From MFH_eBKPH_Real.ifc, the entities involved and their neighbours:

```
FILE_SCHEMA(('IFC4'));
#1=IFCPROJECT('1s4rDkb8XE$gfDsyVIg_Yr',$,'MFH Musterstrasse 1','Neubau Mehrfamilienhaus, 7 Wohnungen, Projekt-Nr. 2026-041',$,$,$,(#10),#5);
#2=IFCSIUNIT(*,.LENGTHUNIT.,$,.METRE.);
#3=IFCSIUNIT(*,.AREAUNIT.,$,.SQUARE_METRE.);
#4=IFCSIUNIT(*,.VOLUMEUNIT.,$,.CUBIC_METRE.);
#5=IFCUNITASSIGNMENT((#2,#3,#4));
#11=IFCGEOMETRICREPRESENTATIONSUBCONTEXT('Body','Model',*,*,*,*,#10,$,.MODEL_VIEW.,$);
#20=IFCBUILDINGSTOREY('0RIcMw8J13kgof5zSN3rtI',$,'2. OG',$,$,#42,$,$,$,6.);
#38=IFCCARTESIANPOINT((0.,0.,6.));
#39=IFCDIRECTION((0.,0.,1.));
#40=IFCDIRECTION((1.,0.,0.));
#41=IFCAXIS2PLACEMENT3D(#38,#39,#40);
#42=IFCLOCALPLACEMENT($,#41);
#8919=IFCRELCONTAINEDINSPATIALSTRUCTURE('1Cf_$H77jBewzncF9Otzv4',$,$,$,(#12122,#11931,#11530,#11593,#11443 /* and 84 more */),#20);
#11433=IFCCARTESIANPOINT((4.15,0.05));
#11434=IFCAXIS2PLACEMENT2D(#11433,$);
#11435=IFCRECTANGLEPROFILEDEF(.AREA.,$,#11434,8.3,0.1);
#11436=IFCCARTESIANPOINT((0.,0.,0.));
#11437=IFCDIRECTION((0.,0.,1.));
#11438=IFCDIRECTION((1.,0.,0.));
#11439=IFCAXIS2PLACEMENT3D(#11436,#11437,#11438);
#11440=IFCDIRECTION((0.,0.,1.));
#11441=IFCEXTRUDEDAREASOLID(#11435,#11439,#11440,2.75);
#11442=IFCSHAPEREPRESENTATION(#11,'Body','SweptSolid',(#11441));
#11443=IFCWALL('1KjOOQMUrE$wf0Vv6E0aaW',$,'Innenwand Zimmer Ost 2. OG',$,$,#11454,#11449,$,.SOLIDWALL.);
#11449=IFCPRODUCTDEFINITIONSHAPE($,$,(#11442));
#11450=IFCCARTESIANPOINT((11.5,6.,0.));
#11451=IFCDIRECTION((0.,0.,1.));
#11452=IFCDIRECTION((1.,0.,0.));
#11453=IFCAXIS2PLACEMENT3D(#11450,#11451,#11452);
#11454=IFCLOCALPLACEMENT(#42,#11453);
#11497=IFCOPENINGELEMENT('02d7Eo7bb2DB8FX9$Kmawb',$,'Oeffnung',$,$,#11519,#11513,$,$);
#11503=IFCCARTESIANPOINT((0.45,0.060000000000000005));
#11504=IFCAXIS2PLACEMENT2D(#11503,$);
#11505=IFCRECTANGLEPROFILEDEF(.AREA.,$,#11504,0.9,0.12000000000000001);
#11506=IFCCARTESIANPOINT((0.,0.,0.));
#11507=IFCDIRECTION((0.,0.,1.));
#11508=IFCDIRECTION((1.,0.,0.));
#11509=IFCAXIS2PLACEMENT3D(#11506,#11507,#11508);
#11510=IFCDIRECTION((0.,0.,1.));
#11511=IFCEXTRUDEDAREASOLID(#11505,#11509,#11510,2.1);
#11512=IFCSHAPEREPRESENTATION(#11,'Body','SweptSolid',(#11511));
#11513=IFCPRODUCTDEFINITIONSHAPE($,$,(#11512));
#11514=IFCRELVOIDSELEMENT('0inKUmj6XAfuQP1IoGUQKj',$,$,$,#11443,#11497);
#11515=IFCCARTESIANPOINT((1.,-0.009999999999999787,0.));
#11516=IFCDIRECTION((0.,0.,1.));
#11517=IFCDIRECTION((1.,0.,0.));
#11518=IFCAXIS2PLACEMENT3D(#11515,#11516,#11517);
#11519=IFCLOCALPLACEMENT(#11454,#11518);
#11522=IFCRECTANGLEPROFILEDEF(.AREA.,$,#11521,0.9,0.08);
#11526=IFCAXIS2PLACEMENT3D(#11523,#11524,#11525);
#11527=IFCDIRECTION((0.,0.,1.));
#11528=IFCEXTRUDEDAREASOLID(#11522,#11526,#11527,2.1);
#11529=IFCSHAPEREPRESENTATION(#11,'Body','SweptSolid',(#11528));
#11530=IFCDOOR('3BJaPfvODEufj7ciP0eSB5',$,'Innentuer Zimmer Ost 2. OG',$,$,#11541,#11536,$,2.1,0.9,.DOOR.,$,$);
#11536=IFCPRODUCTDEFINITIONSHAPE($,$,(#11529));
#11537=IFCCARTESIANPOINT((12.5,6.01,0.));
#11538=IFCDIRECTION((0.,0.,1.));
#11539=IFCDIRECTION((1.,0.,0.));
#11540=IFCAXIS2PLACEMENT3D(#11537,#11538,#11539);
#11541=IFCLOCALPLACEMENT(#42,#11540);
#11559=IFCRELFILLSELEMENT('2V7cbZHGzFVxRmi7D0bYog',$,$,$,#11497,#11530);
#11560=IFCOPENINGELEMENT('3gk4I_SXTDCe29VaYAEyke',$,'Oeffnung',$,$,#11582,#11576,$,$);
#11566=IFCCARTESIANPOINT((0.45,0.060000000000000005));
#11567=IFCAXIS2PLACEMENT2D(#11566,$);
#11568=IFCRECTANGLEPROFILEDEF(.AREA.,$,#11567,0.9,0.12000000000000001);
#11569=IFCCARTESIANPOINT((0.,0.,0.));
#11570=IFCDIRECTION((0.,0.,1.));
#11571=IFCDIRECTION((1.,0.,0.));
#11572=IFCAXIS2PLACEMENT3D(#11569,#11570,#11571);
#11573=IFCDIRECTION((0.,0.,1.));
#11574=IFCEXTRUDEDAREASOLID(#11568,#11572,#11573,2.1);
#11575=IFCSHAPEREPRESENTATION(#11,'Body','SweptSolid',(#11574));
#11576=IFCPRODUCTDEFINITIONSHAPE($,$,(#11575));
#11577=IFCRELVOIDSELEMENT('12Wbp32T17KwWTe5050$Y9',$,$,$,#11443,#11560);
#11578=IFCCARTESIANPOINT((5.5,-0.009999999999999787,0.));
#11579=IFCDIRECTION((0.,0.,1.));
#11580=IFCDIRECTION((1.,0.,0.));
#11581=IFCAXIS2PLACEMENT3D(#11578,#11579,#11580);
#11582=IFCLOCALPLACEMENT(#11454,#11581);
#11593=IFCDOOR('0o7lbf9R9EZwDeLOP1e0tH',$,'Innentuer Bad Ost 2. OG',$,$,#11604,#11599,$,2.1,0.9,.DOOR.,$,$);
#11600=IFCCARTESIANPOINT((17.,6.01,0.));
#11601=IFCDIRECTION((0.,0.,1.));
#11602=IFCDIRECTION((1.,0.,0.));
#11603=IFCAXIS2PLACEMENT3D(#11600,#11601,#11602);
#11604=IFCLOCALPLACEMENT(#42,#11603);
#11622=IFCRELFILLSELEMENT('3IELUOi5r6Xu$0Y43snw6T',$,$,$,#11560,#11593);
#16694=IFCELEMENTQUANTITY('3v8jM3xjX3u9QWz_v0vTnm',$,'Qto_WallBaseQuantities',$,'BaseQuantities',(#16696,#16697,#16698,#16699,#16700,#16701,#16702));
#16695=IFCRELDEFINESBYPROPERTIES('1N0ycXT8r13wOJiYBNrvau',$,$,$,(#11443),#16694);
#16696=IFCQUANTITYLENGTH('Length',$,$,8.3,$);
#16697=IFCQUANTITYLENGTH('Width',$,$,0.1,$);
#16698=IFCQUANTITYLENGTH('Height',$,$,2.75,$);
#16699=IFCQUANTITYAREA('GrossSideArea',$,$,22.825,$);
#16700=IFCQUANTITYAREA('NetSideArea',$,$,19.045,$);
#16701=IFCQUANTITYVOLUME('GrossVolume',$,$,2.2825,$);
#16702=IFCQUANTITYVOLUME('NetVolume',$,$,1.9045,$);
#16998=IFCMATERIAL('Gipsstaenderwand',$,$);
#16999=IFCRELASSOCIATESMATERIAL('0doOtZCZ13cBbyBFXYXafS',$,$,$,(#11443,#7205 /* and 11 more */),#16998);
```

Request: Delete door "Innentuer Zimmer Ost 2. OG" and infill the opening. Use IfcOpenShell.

```python
import ifcopenshell
import ifcopenshell.api.feature
import ifcopenshell.api.pset
import ifcopenshell.api.root
import ifcopenshell.geom
import ifcopenshell.util.element
import ifcopenshell.util.shape
import ifcopenshell.util.unit

model = ifcopenshell.open("MFH_eBKPH_Real.ifc")
area_scale = ifcopenshell.util.unit.calculate_unit_scale(model, "AREAUNIT")
volume_scale = ifcopenshell.util.unit.calculate_unit_scale(model, "VOLUMEUNIT")
settings = ifcopenshell.geom.settings()


def volume(element):
    """Net volume in cubic metres, openings subtracted."""
    shape = ifcopenshell.geom.create_shape(settings, element)
    return ifcopenshell.util.shape.get_volume(shape.geometry)


door = model.by_id(11530)
opening = door.FillsVoids[0].RelatingOpeningElement
wall = opening.VoidsElements[0].RelatingBuildingElement
before = volume(wall)

ifcopenshell.api.root.remove_product(model, product=door)
ifcopenshell.api.feature.remove_feature(model, feature=opening)

after = volume(wall)
thickness = 0.1  # wall thickness in metres

# Update the wall's stored quantities.
qto = model.by_id(ifcopenshell.util.element.get_pset(wall, "Qto_WallBaseQuantities", should_inherit=False)["id"])
ifcopenshell.api.pset.edit_qto(model, qto=qto, properties={
    "NetSideArea": after / thickness / area_scale,
    "NetVolume": after / volume_scale,
})

print(f"wall volume {before:.3f} -> {after:.3f} m3")

model.write("MFH_eBKPH_Real_edited.ifc")
```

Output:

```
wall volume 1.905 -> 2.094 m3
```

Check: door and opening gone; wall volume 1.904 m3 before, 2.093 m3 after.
